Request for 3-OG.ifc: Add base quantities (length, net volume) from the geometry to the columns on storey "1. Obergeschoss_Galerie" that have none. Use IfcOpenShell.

First a look at what the model holds.

```python
import ifcopenshell
import ifcopenshell.util.element
import ifcopenshell.util.unit

model = ifcopenshell.open("3-OG.ifc")
print(model.schema)
for unit_type in ("LENGTHUNIT", "AREAUNIT", "VOLUMEUNIT"):
    print(unit_type, ifcopenshell.util.unit.calculate_unit_scale(model, unit_type))
storey = next(s for s in model.by_type("IfcBuildingStorey") if s.Name == "1. Obergeschoss_Galerie")
columns = [e for e in ifcopenshell.util.element.get_decomposition(storey) if e.is_a("IfcColumn")]
for e in sorted(columns, key=lambda e: e.id()):
    print(e.id(), e.is_a(), e.Name, list(ifcopenshell.util.element.get_psets(e, qtos_only=True)), sep=" | ")
```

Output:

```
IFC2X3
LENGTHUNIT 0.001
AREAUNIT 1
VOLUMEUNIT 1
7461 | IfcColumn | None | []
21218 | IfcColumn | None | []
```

```python
import ifcopenshell
import ifcopenshell.api.pset
import ifcopenshell.geom
import ifcopenshell.util.element
import ifcopenshell.util.shape
import ifcopenshell.util.unit

model = ifcopenshell.open("3-OG.ifc")
unit_scale = ifcopenshell.util.unit.calculate_unit_scale(model)
volume_scale = ifcopenshell.util.unit.calculate_unit_scale(model, "VOLUMEUNIT")
settings = ifcopenshell.geom.settings()

storey = next(s for s in model.by_type("IfcBuildingStorey") if s.Name == "1. Obergeschoss_Galerie")
columns = [e for e in ifcopenshell.util.element.get_decomposition(storey) if e.is_a("IfcColumn")]

for e in sorted(columns, key=lambda e: e.id()):
    if ifcopenshell.util.element.get_psets(e, qtos_only=True, should_inherit=False):
        continue
    # Geometry comes back in metres, in the element's own axes.
    shape = ifcopenshell.geom.create_shape(settings, e)
    values = {
        "Length": ifcopenshell.util.shape.get_z(shape.geometry) / unit_scale,
        "NetVolume": ifcopenshell.util.shape.get_volume(shape.geometry) / volume_scale,
    }
    qto = ifcopenshell.api.pset.add_qto(model, product=e, name="BaseQuantities")
    ifcopenshell.api.pset.edit_qto(model, qto=qto, properties=values)
    print(e.id(), {k: round(v, 3) for k, v in values.items()})

model.write("3-OG_updated.ifc")
```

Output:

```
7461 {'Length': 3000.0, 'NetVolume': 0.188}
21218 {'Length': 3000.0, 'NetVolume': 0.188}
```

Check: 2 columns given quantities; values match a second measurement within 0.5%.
